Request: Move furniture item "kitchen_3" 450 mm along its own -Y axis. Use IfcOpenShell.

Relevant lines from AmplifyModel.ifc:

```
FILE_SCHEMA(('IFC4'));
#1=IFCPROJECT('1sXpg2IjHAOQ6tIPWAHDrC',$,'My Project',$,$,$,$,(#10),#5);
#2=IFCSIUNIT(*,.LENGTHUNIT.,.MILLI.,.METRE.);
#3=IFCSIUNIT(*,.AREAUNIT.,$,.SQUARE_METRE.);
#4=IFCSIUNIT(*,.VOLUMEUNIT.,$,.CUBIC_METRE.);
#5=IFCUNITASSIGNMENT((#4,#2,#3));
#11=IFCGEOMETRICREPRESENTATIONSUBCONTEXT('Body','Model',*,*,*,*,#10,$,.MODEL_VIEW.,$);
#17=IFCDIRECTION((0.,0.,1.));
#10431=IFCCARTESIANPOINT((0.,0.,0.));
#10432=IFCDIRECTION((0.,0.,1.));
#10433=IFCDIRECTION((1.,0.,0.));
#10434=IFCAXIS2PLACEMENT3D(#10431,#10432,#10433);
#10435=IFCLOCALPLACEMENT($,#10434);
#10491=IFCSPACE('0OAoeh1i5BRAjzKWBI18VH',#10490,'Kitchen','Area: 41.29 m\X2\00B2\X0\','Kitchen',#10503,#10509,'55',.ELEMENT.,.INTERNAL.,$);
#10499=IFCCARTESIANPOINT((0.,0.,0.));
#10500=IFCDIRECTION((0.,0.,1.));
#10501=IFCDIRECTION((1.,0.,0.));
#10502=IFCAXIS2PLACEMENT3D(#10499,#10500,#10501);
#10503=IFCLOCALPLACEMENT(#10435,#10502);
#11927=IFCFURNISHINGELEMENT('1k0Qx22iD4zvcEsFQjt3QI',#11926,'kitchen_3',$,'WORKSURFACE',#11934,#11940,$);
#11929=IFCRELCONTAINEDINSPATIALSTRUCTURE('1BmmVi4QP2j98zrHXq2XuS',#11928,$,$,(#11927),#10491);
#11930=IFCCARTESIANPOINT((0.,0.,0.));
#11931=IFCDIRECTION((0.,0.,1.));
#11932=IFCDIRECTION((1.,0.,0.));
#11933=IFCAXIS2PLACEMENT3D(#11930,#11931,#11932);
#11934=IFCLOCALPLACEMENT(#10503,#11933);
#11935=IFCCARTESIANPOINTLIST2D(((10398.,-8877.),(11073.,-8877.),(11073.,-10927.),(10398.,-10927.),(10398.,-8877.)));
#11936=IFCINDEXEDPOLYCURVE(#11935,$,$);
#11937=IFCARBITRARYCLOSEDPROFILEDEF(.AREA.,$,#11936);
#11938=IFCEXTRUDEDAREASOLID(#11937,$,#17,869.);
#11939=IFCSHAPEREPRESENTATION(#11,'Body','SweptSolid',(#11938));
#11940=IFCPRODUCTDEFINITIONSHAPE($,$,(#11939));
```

```python
import ifcopenshell
import ifcopenshell.api.geometry
import ifcopenshell.util.placement

model = ifcopenshell.open("AmplifyModel.ifc")

item = model.by_guid("1k0Qx22iD4zvcEsFQjt3QI")
matrix = ifcopenshell.util.placement.get_local_placement(item.ObjectPlacement)
matrix[:3, 3] -= matrix[:3, 1] * 450.0
ifcopenshell.api.geometry.edit_object_placement(model, product=item, matrix=matrix, is_si=False)

print(ifcopenshell.util.placement.get_local_placement(item.ObjectPlacement).round(3) + 0.0)

model.write("AmplifyModel_v2.ifc")
```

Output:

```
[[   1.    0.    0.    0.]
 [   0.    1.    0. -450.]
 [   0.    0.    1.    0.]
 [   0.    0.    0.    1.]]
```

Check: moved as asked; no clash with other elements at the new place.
